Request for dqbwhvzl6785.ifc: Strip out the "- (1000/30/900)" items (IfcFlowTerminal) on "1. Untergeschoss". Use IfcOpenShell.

First a look at what the model holds.

```python
import ifcopenshell
import ifcopenshell.util.element

model = ifcopenshell.open("dqbwhvzl6785.ifc")
print(model.schema)
storey = next(s for s in model.by_type("IfcBuildingStorey") if s.Name == "1. Untergeschoss")
terminals = [e for e in ifcopenshell.util.element.get_decomposition(storey) if e.is_a("IfcFlowTerminal")]
seen = {}
for e in terminals:
    element_type = ifcopenshell.util.element.get_type(e)
    name = element_type.Name if element_type not in (None, e) else None
    seen[name] = seen.get(name, 0) + 1
for name, count in sorted(seen.items(), key=str):
    print(count, "x", name)
```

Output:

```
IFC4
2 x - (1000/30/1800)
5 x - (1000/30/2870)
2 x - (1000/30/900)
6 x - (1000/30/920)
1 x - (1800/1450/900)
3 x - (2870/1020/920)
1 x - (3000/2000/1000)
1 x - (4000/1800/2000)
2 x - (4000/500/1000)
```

```python
import ifcopenshell
import ifcopenshell.api.root
import ifcopenshell.util.element

model = ifcopenshell.open("dqbwhvzl6785.ifc")

storey = next(s for s in model.by_type("IfcBuildingStorey") if s.Name == "1. Untergeschoss")
terminals = [e for e in ifcopenshell.util.element.get_decomposition(storey) if e.is_a("IfcFlowTerminal")]
targets = [e for e in terminals if (t := ifcopenshell.util.element.get_type(e)) not in (None, e) and t.Name == "- (1000/30/900)"]

for e in targets:
    ifcopenshell.api.root.remove_product(model, product=e)
print(len(targets), "removed")

model.write("dqbwhvzl6785_edited.ifc")
```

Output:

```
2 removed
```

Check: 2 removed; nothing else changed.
